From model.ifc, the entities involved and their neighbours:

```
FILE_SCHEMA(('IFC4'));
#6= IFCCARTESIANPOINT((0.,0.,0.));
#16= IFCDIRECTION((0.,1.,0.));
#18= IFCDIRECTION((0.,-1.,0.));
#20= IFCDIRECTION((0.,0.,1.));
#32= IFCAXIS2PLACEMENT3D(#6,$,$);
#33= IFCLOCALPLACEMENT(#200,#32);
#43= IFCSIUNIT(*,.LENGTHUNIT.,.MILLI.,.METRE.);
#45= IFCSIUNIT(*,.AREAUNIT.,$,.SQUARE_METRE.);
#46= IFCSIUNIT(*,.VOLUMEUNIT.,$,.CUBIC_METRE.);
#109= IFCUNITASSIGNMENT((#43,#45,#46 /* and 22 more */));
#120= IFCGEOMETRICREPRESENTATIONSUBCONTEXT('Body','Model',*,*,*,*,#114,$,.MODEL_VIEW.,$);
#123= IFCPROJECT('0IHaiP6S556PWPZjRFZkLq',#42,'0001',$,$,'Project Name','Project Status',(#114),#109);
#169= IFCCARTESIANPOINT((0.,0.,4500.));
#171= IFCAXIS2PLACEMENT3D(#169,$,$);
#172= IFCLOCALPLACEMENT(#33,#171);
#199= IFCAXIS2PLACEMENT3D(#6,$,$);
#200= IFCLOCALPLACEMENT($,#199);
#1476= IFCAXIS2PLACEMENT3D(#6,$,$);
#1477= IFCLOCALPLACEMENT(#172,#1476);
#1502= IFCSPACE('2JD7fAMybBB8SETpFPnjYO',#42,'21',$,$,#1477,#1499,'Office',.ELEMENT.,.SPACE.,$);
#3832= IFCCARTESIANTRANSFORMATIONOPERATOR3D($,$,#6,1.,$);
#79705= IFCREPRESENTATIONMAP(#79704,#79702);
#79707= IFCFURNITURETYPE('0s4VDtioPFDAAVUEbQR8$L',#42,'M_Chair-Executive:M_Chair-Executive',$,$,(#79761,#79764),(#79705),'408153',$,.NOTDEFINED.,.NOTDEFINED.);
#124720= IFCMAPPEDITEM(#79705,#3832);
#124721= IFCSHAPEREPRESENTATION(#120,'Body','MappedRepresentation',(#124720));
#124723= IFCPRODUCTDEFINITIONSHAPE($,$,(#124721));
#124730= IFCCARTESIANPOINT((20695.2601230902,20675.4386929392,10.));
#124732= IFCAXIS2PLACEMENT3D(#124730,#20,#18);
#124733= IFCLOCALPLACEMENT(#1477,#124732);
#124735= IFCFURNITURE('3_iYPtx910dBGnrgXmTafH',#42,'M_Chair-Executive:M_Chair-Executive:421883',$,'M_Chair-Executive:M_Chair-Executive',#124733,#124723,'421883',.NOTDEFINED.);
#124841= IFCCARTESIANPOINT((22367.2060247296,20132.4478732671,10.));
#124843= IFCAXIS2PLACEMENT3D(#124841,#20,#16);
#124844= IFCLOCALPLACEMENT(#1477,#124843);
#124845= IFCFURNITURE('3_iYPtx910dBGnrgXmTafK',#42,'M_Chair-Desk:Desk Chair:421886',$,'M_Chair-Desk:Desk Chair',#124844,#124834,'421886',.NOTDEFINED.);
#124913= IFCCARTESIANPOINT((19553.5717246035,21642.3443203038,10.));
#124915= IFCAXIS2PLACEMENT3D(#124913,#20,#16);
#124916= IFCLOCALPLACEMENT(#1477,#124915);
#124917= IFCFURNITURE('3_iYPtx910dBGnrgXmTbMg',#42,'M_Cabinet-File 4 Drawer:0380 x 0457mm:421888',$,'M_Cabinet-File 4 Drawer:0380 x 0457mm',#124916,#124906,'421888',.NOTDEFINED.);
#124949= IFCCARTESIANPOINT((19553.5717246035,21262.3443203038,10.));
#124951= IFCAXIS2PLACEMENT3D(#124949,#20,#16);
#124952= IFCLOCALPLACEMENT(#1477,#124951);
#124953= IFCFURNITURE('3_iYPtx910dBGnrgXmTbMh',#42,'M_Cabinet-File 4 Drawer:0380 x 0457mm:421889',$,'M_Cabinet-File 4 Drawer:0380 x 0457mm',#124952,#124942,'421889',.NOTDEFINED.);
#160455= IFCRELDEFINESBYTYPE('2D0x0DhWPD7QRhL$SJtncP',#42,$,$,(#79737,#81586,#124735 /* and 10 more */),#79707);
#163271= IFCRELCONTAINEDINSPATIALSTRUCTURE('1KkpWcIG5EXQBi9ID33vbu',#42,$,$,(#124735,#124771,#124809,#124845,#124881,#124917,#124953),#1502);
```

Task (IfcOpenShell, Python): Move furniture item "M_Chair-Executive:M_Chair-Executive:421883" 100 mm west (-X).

```python
import ifcopenshell
import ifcopenshell.api.geometry
import ifcopenshell.util.placement

model = ifcopenshell.open("model.ifc")

item = model.by_id(124735)
matrix = ifcopenshell.util.placement.get_local_placement(item.ObjectPlacement)
matrix[0, 3] -= 100.0
ifcopenshell.api.geometry.edit_object_placement(model, product=item, matrix=matrix, is_si=False)

print(ifcopenshell.util.placement.get_local_placement(item.ObjectPlacement).round(3) + 0.0)

model.write("model-out.ifc")
```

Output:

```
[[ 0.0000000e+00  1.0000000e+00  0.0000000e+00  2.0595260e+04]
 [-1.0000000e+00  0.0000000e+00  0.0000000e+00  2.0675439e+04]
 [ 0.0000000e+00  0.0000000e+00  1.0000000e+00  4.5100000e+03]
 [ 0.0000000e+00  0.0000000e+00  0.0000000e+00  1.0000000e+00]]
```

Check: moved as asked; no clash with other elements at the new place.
